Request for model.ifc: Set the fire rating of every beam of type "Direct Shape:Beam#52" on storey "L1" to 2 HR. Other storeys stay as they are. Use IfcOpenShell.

First a look at what the model holds.

```python
import ifcopenshell
import ifcopenshell.util.element

model = ifcopenshell.open("model.ifc")
print(model.schema)
storey = next(s for s in model.by_type("IfcBuildingStorey") if s.Name == "L1")
beams = [e for e in ifcopenshell.util.element.get_decomposition(storey) if e.is_a("IfcBeam")]
seen = {}
for e in beams:
    element_type = ifcopenshell.util.element.get_type(e)
    key = (element_type.Name if element_type != e and element_type else None, ifcopenshell.util.element.get_pset(e, "Pset_BeamCommon", "FireRating"))
    seen[key] = seen.get(key, 0) + 1
for (name, value), count in sorted(seen.items(), key=str):
    print(count, "x", name, "|", value)
```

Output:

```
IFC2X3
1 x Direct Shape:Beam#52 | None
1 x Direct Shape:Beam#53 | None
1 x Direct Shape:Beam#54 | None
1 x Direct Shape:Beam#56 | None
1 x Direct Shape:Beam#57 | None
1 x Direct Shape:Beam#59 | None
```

```python
import ifcopenshell
import ifcopenshell.api.pset
import ifcopenshell.util.element

model = ifcopenshell.open("model.ifc")

storey = next(s for s in model.by_type("IfcBuildingStorey") if s.Name == "L1")
beams = [e for e in ifcopenshell.util.element.get_decomposition(storey) if e.is_a("IfcBeam")]

count = 0
for e in beams:
    element_type = ifcopenshell.util.element.get_type(e)
    if element_type in (None, e) or element_type.Name != "Direct Shape:Beam#52":
        continue
    # add_pset returns the element's existing set when there is one.
    pset = ifcopenshell.api.pset.add_pset(model, product=e, name="Pset_BeamCommon")
    ifcopenshell.api.pset.edit_pset(model, pset=pset, properties={"FireRating": "2 HR"})
    count += 1

print(count, "beams updated")

model.write("model_updated.ifc")
```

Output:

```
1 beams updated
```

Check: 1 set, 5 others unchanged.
